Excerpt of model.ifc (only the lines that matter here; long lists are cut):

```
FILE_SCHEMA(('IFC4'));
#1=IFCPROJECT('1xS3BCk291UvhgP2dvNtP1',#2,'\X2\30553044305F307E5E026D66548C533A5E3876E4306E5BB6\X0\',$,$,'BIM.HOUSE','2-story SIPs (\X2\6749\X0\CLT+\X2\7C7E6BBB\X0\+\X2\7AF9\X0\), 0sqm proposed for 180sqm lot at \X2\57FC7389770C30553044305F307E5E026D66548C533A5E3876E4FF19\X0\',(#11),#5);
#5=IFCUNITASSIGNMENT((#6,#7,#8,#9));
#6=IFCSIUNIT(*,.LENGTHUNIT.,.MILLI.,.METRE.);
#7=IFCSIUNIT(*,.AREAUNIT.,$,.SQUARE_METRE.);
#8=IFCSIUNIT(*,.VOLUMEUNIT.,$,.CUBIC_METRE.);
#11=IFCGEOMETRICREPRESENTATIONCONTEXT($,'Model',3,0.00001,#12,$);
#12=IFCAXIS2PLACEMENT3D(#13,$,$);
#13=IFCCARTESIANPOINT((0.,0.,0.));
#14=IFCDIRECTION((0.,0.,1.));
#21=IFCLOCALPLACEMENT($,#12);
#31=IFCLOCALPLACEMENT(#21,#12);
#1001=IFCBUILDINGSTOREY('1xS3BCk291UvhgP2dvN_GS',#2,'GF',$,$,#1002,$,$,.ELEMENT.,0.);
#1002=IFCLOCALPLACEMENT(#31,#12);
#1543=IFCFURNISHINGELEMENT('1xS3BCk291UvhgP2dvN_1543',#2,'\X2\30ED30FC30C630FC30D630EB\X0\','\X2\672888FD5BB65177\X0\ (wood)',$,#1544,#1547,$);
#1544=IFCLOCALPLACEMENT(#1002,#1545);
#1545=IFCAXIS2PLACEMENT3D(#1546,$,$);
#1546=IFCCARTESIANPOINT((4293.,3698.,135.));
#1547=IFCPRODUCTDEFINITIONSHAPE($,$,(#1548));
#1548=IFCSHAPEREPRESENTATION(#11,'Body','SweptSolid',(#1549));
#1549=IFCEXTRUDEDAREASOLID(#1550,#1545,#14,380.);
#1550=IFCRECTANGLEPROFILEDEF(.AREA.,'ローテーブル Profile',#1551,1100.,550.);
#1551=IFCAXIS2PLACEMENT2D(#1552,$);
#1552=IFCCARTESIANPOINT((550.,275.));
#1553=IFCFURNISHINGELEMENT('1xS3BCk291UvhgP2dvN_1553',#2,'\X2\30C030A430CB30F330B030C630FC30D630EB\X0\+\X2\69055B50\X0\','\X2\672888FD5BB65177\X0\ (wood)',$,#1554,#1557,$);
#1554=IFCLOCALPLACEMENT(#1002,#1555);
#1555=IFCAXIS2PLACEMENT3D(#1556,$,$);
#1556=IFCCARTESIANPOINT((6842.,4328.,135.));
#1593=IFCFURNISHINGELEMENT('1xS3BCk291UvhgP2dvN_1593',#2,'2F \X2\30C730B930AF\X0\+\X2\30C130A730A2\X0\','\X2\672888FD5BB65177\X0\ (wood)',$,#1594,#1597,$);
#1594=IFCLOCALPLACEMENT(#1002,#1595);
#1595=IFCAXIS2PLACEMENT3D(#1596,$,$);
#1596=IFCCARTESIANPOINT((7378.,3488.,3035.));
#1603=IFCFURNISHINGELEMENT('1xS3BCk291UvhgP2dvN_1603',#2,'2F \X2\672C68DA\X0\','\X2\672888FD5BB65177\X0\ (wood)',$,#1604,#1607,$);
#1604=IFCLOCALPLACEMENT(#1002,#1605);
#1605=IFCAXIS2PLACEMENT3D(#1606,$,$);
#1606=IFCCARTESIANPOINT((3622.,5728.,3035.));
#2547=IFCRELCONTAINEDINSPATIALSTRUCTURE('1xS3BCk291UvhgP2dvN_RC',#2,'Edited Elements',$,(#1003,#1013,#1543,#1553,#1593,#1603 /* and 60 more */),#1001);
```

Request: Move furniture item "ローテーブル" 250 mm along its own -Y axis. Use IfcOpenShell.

```python
import ifcopenshell
import ifcopenshell.api.geometry
import ifcopenshell.util.placement
import ifcopenshell.util.unit

model = ifcopenshell.open("model.ifc")
unit_scale = ifcopenshell.util.unit.calculate_unit_scale(model)

item = model.by_guid("1xS3BCk291UvhgP2dvN_1543")
matrix = ifcopenshell.util.placement.get_local_placement(item.ObjectPlacement)
matrix[:3, 3] -= matrix[:3, 1] * 0.25 / unit_scale
ifcopenshell.api.geometry.edit_object_placement(model, product=item, matrix=matrix, is_si=False)

print(ifcopenshell.util.placement.get_local_placement(item.ObjectPlacement).round(3) + 0.0)

model.write("model_edited.ifc")
```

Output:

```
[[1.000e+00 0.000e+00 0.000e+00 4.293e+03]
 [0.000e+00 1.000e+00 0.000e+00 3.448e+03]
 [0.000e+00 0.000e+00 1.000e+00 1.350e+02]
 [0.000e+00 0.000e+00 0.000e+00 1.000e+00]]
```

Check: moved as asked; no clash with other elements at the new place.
